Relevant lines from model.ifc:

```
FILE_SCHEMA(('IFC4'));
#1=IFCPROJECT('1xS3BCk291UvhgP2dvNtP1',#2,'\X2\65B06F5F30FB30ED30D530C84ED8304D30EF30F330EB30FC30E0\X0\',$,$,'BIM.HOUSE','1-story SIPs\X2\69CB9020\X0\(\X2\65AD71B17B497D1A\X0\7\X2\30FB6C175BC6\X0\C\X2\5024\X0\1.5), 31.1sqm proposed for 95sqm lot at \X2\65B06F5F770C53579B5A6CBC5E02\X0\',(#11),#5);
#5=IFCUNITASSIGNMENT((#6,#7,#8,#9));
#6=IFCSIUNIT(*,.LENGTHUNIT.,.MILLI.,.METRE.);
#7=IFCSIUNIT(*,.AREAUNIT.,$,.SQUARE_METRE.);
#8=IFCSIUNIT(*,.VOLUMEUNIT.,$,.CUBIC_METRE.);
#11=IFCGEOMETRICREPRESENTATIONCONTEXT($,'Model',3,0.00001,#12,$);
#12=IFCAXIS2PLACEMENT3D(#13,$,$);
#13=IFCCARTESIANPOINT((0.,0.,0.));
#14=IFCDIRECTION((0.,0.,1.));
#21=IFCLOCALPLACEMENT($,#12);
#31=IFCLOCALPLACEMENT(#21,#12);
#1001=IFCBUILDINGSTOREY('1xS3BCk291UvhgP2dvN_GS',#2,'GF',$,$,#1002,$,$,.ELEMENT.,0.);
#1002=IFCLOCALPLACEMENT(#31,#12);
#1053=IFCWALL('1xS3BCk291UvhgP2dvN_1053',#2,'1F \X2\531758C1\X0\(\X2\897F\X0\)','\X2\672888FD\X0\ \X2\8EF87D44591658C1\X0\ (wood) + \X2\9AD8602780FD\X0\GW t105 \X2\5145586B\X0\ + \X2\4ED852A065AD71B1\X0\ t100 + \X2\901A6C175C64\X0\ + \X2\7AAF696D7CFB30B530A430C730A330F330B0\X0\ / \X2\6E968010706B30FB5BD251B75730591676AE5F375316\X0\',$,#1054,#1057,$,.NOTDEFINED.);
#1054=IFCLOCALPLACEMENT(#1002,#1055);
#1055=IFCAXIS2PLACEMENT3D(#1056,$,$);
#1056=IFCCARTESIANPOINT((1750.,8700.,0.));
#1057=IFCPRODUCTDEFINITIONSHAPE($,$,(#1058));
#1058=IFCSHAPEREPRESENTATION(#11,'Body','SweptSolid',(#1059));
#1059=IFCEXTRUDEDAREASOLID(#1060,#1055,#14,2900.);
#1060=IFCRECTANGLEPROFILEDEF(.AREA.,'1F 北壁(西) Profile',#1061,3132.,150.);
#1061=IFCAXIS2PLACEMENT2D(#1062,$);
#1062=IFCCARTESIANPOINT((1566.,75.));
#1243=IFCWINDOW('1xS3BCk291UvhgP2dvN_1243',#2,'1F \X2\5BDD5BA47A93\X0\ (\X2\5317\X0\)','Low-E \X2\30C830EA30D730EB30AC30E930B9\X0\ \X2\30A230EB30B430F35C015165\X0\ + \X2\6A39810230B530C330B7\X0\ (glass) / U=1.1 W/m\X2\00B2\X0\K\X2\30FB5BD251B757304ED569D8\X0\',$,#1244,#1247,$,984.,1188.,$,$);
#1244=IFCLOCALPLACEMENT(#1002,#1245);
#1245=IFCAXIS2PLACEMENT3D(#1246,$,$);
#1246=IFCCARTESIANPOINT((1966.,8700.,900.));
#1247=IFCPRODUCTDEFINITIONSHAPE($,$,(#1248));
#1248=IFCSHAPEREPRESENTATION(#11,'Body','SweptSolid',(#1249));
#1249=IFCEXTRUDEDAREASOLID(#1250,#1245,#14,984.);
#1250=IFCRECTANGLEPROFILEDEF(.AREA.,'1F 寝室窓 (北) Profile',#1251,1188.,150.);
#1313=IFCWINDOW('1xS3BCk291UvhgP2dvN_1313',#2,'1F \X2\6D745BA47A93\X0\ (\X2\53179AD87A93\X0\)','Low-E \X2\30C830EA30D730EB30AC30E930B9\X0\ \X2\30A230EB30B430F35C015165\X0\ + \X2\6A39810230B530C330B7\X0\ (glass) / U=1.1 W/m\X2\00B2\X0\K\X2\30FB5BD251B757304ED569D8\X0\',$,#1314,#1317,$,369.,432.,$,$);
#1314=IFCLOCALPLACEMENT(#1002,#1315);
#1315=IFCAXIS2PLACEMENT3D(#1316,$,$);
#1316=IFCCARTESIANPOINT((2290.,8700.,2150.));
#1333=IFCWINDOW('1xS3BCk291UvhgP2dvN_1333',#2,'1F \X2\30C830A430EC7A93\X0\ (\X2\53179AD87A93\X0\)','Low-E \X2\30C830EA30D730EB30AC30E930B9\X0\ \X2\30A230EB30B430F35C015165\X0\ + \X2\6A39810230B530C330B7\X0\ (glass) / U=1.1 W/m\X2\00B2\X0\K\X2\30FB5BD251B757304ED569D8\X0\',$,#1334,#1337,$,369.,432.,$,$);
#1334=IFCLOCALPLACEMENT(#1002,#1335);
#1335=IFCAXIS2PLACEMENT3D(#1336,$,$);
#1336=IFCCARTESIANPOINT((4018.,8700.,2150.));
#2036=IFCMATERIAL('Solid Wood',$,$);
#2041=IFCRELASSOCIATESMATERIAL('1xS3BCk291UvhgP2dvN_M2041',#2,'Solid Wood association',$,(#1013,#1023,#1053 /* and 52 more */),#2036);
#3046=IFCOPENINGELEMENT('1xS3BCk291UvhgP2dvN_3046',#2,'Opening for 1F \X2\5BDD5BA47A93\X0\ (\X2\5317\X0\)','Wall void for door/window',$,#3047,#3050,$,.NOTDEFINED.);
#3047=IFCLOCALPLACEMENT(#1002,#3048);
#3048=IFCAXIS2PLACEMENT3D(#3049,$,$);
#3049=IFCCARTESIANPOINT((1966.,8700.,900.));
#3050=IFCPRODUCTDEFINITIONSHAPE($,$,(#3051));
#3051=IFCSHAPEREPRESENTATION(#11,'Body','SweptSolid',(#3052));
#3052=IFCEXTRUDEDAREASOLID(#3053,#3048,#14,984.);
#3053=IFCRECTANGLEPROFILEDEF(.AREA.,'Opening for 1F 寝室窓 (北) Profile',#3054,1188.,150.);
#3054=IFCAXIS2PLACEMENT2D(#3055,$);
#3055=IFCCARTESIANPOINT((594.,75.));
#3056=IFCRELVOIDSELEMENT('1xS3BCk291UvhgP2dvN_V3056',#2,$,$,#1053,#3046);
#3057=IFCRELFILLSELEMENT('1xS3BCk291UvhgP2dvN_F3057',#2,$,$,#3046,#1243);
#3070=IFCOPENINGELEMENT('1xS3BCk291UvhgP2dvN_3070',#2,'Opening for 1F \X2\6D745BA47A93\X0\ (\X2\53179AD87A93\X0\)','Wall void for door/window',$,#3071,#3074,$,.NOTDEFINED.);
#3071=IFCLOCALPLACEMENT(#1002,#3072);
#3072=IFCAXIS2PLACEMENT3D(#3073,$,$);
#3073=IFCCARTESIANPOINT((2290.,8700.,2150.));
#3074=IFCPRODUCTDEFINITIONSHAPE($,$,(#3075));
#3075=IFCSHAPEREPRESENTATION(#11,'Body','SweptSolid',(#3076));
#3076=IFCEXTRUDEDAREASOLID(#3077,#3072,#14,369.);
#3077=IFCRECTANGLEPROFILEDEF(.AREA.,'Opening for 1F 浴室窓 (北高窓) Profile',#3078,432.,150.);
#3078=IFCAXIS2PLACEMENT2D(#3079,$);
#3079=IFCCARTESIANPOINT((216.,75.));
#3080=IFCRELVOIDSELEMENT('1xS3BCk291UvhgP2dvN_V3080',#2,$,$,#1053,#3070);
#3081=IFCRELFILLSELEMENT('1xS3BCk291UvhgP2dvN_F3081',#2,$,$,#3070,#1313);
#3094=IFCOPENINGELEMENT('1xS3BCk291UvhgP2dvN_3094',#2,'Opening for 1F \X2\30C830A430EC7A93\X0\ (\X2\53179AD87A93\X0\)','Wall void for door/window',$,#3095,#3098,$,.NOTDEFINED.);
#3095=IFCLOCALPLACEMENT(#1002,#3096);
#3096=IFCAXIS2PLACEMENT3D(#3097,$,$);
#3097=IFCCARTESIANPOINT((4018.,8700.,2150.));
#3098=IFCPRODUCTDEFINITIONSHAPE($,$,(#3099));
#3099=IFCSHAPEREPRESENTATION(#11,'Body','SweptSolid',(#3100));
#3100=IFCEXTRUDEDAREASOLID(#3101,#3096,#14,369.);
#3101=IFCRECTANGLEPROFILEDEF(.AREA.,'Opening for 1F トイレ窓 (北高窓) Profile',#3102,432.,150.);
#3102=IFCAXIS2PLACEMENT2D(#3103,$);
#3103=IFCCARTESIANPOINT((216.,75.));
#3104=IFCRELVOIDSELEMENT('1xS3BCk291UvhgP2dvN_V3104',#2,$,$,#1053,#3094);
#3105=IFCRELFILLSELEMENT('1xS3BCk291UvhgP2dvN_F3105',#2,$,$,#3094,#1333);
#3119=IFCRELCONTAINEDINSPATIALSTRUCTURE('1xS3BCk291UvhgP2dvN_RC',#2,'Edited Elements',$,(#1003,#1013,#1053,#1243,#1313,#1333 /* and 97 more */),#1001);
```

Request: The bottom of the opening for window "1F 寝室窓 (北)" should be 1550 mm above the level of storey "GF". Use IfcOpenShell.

```python
import numpy as np
import ifcopenshell
import ifcopenshell.api.geometry
import ifcopenshell.geom
import ifcopenshell.util.element
import ifcopenshell.util.placement
import ifcopenshell.util.shape
import ifcopenshell.util.unit

model = ifcopenshell.open("model.ifc")
unit_scale = ifcopenshell.util.unit.calculate_unit_scale(model)

window = model.by_id(1243)
opening = window.FillsVoids[0].RelatingOpeningElement
storey = ifcopenshell.util.element.get_container(window, ifc_class="IfcBuildingStorey")
level = ifcopenshell.util.placement.get_local_placement(storey.ObjectPlacement)[2, 3]

# The opening's origin need not be at the sill, so measure its lowest point.
shape = ifcopenshell.geom.create_shape(ifcopenshell.geom.settings(), opening)
bottom = ifcopenshell.util.shape.get_shape_bottom_elevation(shape, shape.geometry) / unit_scale
dz = level + 1.55 / unit_scale - bottom

shift = np.array([0.0, 0.0, dz])
# The window is not placed relative to its opening, so move both.
for product in (opening, window):
    matrix = ifcopenshell.util.placement.get_local_placement(product.ObjectPlacement)
    matrix[:3, 3] += shift
    ifcopenshell.api.geometry.edit_object_placement(model, product=product, matrix=matrix, is_si=False)

print(f"moved by {dz * unit_scale:+.3f} m")

model.write("model_edited.ifc")
```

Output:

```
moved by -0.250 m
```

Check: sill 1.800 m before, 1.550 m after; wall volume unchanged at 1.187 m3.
